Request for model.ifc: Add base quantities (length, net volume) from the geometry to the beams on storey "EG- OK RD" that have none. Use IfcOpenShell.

First a look at what the model holds.

```python
import ifcopenshell
import ifcopenshell.util.element
import ifcopenshell.util.unit

model = ifcopenshell.open("model.ifc")
print(model.schema)
for unit_type in ("LENGTHUNIT", "AREAUNIT", "VOLUMEUNIT"):
    print(unit_type, ifcopenshell.util.unit.calculate_unit_scale(model, unit_type))
storey = next(s for s in model.by_type("IfcBuildingStorey") if s.Name == "EG- OK RD")
beams = [e for e in ifcopenshell.util.element.get_decomposition(storey) if e.is_a("IfcBeam")]
for e in sorted(beams, key=lambda e: e.id()):
    print(e.id(), e.is_a(), e.Name, list(ifcopenshell.util.element.get_psets(e, qtos_only=True)), sep=" | ")
```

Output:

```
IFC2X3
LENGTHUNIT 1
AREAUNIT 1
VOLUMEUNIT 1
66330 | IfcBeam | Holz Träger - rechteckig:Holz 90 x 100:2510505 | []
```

```python
import ifcopenshell
import ifcopenshell.api.pset
import ifcopenshell.geom
import ifcopenshell.util.element
import ifcopenshell.util.shape
import ifcopenshell.util.unit

model = ifcopenshell.open("model.ifc")
unit_scale = ifcopenshell.util.unit.calculate_unit_scale(model)
volume_scale = ifcopenshell.util.unit.calculate_unit_scale(model, "VOLUMEUNIT")
settings = ifcopenshell.geom.settings()

storey = next(s for s in model.by_type("IfcBuildingStorey") if s.Name == "EG- OK RD")
beams = [e for e in ifcopenshell.util.element.get_decomposition(storey) if e.is_a("IfcBeam")]

for e in sorted(beams, key=lambda e: e.id()):
    if ifcopenshell.util.element.get_psets(e, qtos_only=True, should_inherit=False):
        continue
    # Geometry comes back in metres, in the element's own axes.
    shape = ifcopenshell.geom.create_shape(settings, e)
    values = {
        "Length": ifcopenshell.util.shape.get_max_xyz(shape.geometry) / unit_scale,
        "NetVolume": ifcopenshell.util.shape.get_volume(shape.geometry) / volume_scale,
    }
    qto = ifcopenshell.api.pset.add_qto(model, product=e, name="BaseQuantities")
    ifcopenshell.api.pset.edit_qto(model, qto=qto, properties=values)
    print(e.id(), {k: round(v, 3) for k, v in values.items()})

model.write("model_v2.ifc")
```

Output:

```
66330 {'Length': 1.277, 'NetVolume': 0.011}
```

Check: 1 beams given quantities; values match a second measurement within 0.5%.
